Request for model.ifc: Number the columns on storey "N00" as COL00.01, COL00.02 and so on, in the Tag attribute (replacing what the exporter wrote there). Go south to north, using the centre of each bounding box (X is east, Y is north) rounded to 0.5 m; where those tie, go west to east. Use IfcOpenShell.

First a look at what the model holds.

```python
import ifcopenshell
import ifcopenshell.util.element
import ifcopenshell.util.placement

model = ifcopenshell.open("model.ifc")
print(model.schema)
storey = next(s for s in model.by_type("IfcBuildingStorey") if s.Name == "N00")
columns = [e for e in ifcopenshell.util.element.get_decomposition(storey) if e.is_a("IfcColumn")]
for e in sorted(columns, key=lambda e: e.id()):
    origin = ifcopenshell.util.placement.get_local_placement(e.ObjectPlacement)[:3, 3]
    print(e.id(), e.Tag, e.Name, origin.round(2) + 0.0, sep=" | ")
```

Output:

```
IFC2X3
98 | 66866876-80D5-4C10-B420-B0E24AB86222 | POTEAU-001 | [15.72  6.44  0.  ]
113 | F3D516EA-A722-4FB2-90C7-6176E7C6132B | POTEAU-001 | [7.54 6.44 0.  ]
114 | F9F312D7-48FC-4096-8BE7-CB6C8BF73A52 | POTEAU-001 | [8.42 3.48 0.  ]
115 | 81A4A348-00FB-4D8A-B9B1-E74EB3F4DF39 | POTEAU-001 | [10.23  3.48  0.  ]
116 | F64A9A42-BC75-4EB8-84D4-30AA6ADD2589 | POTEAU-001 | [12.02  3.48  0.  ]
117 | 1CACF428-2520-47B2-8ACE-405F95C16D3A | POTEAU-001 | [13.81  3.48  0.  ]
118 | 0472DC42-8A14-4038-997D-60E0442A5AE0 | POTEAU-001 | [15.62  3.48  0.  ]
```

```python
import ifcopenshell
import ifcopenshell.geom
import ifcopenshell.util.element
import ifcopenshell.util.shape

model = ifcopenshell.open("model.ifc")
settings = ifcopenshell.geom.settings()
settings.set("use-world-coords", True)


def centre(element):
    shape = ifcopenshell.geom.create_shape(settings, element)
    return ifcopenshell.util.shape.get_bbox_centroid(shape.geometry)


storey = next(s for s in model.by_type("IfcBuildingStorey") if s.Name == "N00")
columns = [e for e in ifcopenshell.util.element.get_decomposition(storey) if e.is_a("IfcColumn")]

# Insertion points can sit at a corner or the storey origin, so sort by the geometry (in metres).
centres = {e: centre(e) for e in columns}
columns.sort(key=lambda e: (round(centres[e][1] / 0.5), centres[e][0]))

for i, e in enumerate(columns, start=1):
    number = f"COL00.{i:02d}"
    e.Tag = number
    print(e.id(), number)

model.write("model_v2.ifc")
```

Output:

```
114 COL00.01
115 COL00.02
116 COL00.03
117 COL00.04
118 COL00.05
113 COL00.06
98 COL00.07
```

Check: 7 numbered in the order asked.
